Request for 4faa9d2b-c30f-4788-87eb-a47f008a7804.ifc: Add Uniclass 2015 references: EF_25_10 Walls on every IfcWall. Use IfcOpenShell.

First a look at what the model holds.

```python
import ifcopenshell

model = ifcopenshell.open("4faa9d2b-c30f-4788-87eb-a47f008a7804.ifc")
print(model.schema)
print("classifications:", [c.Name for c in model.by_type("IfcClassification")])
for ifc_class in ("IfcDoor", "IfcRoof", "IfcStair", "IfcWall", "IfcWindow"):
    print(ifc_class, len(model.by_type(ifc_class)))
```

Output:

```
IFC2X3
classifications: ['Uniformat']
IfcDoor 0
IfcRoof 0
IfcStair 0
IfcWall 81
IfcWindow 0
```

```python
import ifcopenshell
import ifcopenshell.api.classification

model = ifcopenshell.open("4faa9d2b-c30f-4788-87eb-a47f008a7804.ifc")

# IFC2X3 requires Source and Edition and has no link from the project to the system.
system = model.create_entity("IfcClassification", Source="NBS", Edition="2015", Name="Uniclass 2015")

codes = {
    "IfcWall": ("EF_25_10", "Walls"),
}
for ifc_class, (code, name) in codes.items():
    products = model.by_type(ifc_class)
    ifcopenshell.api.classification.add_reference(
        model, products=products, classification=system, identification=code, name=name
    )
    print(code, len(products))

model.write("4faa9d2b-c30f-4788-87eb-a47f008a7804_updated.ifc")
```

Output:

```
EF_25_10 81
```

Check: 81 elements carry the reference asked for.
